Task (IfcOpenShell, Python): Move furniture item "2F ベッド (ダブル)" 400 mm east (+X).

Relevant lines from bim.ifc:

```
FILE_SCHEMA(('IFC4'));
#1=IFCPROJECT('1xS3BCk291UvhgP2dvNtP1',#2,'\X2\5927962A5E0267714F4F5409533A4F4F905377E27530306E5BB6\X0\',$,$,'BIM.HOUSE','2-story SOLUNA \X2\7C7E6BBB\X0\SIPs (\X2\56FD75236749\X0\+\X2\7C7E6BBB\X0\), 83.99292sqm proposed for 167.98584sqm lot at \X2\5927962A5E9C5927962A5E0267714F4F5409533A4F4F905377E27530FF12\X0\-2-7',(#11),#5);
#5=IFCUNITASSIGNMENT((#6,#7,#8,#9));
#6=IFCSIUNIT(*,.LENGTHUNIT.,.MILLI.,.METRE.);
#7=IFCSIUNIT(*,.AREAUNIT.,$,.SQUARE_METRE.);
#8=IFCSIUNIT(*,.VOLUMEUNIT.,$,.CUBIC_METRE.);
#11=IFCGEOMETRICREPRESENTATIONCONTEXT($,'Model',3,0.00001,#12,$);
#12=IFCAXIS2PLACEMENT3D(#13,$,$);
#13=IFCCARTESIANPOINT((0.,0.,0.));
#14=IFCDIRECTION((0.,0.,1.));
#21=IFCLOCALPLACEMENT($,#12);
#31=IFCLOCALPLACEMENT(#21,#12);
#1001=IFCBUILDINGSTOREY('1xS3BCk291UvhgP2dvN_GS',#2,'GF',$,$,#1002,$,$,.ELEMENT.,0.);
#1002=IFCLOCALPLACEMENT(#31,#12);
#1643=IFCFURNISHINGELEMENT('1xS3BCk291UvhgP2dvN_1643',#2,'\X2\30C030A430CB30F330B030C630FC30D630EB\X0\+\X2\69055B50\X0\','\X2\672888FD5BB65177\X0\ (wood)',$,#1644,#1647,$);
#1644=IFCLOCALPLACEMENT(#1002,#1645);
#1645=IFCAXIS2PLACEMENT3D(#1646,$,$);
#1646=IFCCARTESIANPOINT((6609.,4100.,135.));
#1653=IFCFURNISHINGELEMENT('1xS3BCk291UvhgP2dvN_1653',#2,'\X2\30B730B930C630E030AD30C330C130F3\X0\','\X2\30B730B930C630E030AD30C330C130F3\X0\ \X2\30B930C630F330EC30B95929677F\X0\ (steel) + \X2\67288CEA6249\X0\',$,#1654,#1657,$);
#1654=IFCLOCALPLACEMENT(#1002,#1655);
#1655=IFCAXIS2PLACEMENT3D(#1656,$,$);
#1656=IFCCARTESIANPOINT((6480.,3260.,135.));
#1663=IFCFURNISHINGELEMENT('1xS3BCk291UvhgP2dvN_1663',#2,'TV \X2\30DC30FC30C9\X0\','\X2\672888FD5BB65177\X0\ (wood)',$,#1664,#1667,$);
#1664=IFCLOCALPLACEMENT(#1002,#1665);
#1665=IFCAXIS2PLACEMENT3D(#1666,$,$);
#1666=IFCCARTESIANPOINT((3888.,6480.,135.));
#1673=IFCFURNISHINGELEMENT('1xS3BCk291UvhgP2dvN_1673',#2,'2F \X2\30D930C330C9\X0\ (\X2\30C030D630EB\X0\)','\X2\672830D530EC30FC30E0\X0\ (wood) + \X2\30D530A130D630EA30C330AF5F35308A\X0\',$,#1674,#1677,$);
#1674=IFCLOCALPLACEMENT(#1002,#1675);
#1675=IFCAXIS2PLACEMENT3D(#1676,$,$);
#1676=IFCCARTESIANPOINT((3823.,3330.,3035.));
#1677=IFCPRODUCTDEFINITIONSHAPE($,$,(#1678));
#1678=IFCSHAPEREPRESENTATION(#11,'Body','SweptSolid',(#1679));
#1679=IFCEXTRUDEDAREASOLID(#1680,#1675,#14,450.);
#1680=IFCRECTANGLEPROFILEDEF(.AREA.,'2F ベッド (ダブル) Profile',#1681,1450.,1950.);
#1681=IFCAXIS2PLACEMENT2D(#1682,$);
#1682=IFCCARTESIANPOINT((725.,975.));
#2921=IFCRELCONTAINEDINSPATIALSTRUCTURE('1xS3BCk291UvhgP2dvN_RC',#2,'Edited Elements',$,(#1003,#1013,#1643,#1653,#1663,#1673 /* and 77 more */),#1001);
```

```python
import ifcopenshell
import ifcopenshell.api.geometry
import ifcopenshell.util.placement
import ifcopenshell.util.unit

model = ifcopenshell.open("bim.ifc")
unit_scale = ifcopenshell.util.unit.calculate_unit_scale(model)

item = model.by_guid("1xS3BCk291UvhgP2dvN_1673")
matrix = ifcopenshell.util.placement.get_local_placement(item.ObjectPlacement)
matrix[0, 3] += 0.4 / unit_scale
ifcopenshell.api.geometry.edit_object_placement(model, product=item, matrix=matrix, is_si=False)

print(ifcopenshell.util.placement.get_local_placement(item.ObjectPlacement).round(3) + 0.0)

model.write("bim-out.ifc")
```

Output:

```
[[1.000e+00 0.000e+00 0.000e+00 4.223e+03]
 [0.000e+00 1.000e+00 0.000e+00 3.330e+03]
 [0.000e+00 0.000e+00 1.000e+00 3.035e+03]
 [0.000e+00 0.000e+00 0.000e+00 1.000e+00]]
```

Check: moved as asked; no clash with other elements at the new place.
